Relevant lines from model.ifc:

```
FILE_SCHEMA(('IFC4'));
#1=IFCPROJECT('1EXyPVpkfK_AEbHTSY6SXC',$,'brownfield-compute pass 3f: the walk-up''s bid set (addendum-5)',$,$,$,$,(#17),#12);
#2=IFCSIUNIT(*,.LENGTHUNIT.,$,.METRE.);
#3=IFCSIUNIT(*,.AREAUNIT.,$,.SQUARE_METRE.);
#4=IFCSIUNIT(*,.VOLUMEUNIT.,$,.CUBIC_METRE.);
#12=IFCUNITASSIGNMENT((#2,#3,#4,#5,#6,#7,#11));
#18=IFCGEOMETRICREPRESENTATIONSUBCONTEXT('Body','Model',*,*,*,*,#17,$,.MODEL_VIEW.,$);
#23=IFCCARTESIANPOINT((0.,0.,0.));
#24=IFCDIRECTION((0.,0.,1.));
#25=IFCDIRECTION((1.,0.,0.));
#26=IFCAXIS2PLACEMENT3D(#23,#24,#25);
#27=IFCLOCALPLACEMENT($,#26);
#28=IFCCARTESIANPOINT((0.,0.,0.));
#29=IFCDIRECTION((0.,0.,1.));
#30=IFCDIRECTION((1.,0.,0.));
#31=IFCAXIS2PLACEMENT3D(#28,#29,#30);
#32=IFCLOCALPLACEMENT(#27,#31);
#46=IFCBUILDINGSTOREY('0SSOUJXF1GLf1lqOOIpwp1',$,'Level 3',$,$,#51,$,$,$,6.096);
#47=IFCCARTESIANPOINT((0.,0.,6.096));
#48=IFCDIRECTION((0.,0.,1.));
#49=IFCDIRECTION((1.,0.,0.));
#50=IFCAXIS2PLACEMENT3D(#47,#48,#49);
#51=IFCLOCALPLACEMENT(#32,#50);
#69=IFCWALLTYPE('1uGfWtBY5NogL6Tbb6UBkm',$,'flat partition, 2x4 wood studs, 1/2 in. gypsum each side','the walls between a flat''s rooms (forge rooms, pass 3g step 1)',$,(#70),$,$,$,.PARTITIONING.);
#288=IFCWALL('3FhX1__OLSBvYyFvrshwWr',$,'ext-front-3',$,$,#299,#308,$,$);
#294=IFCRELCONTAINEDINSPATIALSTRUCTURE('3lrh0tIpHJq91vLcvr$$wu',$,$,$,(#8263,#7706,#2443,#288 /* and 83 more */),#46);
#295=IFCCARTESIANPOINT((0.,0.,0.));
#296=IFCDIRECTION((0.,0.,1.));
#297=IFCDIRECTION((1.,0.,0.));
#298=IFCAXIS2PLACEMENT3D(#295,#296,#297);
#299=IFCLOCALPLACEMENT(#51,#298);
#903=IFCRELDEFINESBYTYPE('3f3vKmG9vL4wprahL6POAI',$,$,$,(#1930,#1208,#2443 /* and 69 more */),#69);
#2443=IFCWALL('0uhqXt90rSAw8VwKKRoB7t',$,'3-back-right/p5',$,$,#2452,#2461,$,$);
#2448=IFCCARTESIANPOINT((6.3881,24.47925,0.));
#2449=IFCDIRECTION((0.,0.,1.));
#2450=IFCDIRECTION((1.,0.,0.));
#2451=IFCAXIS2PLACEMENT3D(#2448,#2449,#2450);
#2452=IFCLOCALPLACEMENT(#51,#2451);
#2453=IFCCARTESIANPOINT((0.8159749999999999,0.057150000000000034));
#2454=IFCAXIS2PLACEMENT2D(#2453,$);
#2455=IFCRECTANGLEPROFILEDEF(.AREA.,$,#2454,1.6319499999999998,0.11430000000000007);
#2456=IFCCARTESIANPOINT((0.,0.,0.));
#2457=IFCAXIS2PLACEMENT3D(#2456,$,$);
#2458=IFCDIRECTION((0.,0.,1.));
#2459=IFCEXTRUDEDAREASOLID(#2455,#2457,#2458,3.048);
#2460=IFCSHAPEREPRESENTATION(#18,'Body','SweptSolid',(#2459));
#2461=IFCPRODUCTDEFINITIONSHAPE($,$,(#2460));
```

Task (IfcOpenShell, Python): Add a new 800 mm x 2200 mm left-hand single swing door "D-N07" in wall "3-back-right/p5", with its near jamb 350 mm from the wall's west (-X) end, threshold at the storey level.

```python
import numpy as np
import ifcopenshell
import ifcopenshell.api.feature
import ifcopenshell.api.geometry
import ifcopenshell.api.root
import ifcopenshell.api.spatial
import ifcopenshell.geom
import ifcopenshell.util.element
import ifcopenshell.util.placement
import ifcopenshell.util.representation
import ifcopenshell.util.shape
import ifcopenshell.util.unit

model = ifcopenshell.open("model.ifc")
unit_scale = ifcopenshell.util.unit.calculate_unit_scale(model)
settings = ifcopenshell.geom.settings()


def volume(element):
    """Net volume in cubic metres, openings subtracted."""
    shape = ifcopenshell.geom.create_shape(settings, element)
    return ifcopenshell.util.shape.get_volume(shape.geometry)


wall = model.by_id(2443)
storey = ifcopenshell.util.element.get_container(wall, ifc_class="IfcBuildingStorey")
context = ifcopenshell.util.representation.get_context(model, "Model", "Body", "MODEL_VIEW")
before = volume(wall)

width, height, from_end, sill = 0.8, 2.2, 0.35, 0.0  # metres

# The wall runs along its own X axis, and the end named is its -X end.
wall_shape = ifcopenshell.geom.create_shape(settings, wall)
x, y, z = ifcopenshell.util.shape.get_vertices(wall_shape.geometry).T
start = x.min() + from_end
face, thickness = float(y.min()), float(y.max() - y.min())
wall_matrix = ifcopenshell.util.placement.get_local_placement(wall.ObjectPlacement)
level = ifcopenshell.util.placement.get_local_placement(storey.ObjectPlacement)[2, 3]


def in_wall(x, y):
    """Placement at x, y metres in the wall's axes, at sill height."""
    matrix = wall_matrix.copy()
    matrix[:, 3] = wall_matrix @ np.array([x / unit_scale, y / unit_scale, 0.0, 1.0])
    matrix[2, 3] = level + sill / unit_scale
    return matrix


# Opening: a box that overshoots both wall faces by 50 mm.
opening = ifcopenshell.api.root.create_entity(model, ifc_class="IfcOpeningElement", predefined_type="OPENING")
box = ifcopenshell.api.geometry.add_wall_representation(
    model, context=context, length=width, height=height, thickness=thickness + 0.1
)
ifcopenshell.api.geometry.assign_representation(model, product=opening, representation=box)
ifcopenshell.api.geometry.edit_object_placement(model, product=opening, matrix=in_wall(start, face - 0.05), is_si=False)
ifcopenshell.api.feature.add_feature(model, feature=opening, element=wall)

door = ifcopenshell.api.root.create_entity(model, ifc_class="IfcDoor", name="D-N07", predefined_type="DOOR")
door.OverallWidth, door.OverallHeight = width / unit_scale, height / unit_scale
door.OperationType = "SINGLE_SWING_LEFT"
body = ifcopenshell.api.geometry.add_door_representation(
    model,
    context=context,
    overall_width=door.OverallWidth,
    overall_height=door.OverallHeight,
    operation_type="SINGLE_SWING_LEFT",
    lining_properties={"LiningDepth": thickness / unit_scale, "ThresholdDepth": thickness / unit_scale},
)
ifcopenshell.api.geometry.assign_representation(model, product=door, representation=body)
ifcopenshell.api.spatial.assign_container(model, products=[door], relating_structure=storey)
ifcopenshell.api.feature.add_filling(model, opening=opening, element=door)

# The lining spans the wall, so the door starts at the wall face.
ifcopenshell.api.geometry.edit_object_placement(model, product=door, matrix=in_wall(start, face), is_si=False)

after = volume(wall)

print(f"wall volume {before:.3f} -> {after:.3f} m3")

model.write("model-out.ifc")
```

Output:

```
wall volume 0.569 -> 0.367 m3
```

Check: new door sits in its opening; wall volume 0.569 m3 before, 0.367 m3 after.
